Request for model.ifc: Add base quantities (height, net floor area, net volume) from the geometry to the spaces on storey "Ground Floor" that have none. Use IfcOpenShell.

First a look at what the model holds.

```python
import ifcopenshell
import ifcopenshell.util.element
import ifcopenshell.util.unit

model = ifcopenshell.open("model.ifc")
print(model.schema)
for unit_type in ("LENGTHUNIT", "AREAUNIT", "VOLUMEUNIT"):
    print(unit_type, ifcopenshell.util.unit.calculate_unit_scale(model, unit_type))
storey = next(s for s in model.by_type("IfcBuildingStorey") if s.Name == "Ground Floor")
spaces = [e for e in ifcopenshell.util.element.get_decomposition(storey) if e.is_a("IfcSpace")]
for e in sorted(spaces, key=lambda e: e.id()):
    print(e.id(), e.is_a(), e.Name, list(ifcopenshell.util.element.get_psets(e, qtos_only=True)), sep=" | ")
```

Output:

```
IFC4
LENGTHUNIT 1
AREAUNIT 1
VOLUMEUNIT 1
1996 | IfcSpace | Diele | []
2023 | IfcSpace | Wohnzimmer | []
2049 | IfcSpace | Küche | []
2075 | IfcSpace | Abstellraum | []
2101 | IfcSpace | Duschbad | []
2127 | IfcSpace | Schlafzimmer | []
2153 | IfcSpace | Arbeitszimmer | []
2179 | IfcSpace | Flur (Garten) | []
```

```python
import ifcopenshell
import ifcopenshell.api.pset
import ifcopenshell.geom
import ifcopenshell.util.element
import ifcopenshell.util.shape
import ifcopenshell.util.unit

model = ifcopenshell.open("model.ifc")
unit_scale = ifcopenshell.util.unit.calculate_unit_scale(model)
area_scale = ifcopenshell.util.unit.calculate_unit_scale(model, "AREAUNIT")
volume_scale = ifcopenshell.util.unit.calculate_unit_scale(model, "VOLUMEUNIT")
settings = ifcopenshell.geom.settings()

storey = next(s for s in model.by_type("IfcBuildingStorey") if s.Name == "Ground Floor")
spaces = [e for e in ifcopenshell.util.element.get_decomposition(storey) if e.is_a("IfcSpace")]

for e in sorted(spaces, key=lambda e: e.id()):
    if ifcopenshell.util.element.get_psets(e, qtos_only=True, should_inherit=False):
        continue
    # Geometry comes back in metres, in the element's own axes.
    shape = ifcopenshell.geom.create_shape(settings, e)
    values = {
        "Height": ifcopenshell.util.shape.get_z(shape.geometry) / unit_scale,
        "NetFloorArea": ifcopenshell.util.shape.get_footprint_area(shape.geometry) / area_scale,
        "NetVolume": ifcopenshell.util.shape.get_volume(shape.geometry) / volume_scale,
    }
    qto = ifcopenshell.api.pset.add_qto(model, product=e, name="Qto_SpaceBaseQuantities")
    ifcopenshell.api.pset.edit_qto(model, qto=qto, properties=values)
    print(e.id(), {k: round(v, 3) for k, v in values.items()})

model.write("model_v2.ifc")
```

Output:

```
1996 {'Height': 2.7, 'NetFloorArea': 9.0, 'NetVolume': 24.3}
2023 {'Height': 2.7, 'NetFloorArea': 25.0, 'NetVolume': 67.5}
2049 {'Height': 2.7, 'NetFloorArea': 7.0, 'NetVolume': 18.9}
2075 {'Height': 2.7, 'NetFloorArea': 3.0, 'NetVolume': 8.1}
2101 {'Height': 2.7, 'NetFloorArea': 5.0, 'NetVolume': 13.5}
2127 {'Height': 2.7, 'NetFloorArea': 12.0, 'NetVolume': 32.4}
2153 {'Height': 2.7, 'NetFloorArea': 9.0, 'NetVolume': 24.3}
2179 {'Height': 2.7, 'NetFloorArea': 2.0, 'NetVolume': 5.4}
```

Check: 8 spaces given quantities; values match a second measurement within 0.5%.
